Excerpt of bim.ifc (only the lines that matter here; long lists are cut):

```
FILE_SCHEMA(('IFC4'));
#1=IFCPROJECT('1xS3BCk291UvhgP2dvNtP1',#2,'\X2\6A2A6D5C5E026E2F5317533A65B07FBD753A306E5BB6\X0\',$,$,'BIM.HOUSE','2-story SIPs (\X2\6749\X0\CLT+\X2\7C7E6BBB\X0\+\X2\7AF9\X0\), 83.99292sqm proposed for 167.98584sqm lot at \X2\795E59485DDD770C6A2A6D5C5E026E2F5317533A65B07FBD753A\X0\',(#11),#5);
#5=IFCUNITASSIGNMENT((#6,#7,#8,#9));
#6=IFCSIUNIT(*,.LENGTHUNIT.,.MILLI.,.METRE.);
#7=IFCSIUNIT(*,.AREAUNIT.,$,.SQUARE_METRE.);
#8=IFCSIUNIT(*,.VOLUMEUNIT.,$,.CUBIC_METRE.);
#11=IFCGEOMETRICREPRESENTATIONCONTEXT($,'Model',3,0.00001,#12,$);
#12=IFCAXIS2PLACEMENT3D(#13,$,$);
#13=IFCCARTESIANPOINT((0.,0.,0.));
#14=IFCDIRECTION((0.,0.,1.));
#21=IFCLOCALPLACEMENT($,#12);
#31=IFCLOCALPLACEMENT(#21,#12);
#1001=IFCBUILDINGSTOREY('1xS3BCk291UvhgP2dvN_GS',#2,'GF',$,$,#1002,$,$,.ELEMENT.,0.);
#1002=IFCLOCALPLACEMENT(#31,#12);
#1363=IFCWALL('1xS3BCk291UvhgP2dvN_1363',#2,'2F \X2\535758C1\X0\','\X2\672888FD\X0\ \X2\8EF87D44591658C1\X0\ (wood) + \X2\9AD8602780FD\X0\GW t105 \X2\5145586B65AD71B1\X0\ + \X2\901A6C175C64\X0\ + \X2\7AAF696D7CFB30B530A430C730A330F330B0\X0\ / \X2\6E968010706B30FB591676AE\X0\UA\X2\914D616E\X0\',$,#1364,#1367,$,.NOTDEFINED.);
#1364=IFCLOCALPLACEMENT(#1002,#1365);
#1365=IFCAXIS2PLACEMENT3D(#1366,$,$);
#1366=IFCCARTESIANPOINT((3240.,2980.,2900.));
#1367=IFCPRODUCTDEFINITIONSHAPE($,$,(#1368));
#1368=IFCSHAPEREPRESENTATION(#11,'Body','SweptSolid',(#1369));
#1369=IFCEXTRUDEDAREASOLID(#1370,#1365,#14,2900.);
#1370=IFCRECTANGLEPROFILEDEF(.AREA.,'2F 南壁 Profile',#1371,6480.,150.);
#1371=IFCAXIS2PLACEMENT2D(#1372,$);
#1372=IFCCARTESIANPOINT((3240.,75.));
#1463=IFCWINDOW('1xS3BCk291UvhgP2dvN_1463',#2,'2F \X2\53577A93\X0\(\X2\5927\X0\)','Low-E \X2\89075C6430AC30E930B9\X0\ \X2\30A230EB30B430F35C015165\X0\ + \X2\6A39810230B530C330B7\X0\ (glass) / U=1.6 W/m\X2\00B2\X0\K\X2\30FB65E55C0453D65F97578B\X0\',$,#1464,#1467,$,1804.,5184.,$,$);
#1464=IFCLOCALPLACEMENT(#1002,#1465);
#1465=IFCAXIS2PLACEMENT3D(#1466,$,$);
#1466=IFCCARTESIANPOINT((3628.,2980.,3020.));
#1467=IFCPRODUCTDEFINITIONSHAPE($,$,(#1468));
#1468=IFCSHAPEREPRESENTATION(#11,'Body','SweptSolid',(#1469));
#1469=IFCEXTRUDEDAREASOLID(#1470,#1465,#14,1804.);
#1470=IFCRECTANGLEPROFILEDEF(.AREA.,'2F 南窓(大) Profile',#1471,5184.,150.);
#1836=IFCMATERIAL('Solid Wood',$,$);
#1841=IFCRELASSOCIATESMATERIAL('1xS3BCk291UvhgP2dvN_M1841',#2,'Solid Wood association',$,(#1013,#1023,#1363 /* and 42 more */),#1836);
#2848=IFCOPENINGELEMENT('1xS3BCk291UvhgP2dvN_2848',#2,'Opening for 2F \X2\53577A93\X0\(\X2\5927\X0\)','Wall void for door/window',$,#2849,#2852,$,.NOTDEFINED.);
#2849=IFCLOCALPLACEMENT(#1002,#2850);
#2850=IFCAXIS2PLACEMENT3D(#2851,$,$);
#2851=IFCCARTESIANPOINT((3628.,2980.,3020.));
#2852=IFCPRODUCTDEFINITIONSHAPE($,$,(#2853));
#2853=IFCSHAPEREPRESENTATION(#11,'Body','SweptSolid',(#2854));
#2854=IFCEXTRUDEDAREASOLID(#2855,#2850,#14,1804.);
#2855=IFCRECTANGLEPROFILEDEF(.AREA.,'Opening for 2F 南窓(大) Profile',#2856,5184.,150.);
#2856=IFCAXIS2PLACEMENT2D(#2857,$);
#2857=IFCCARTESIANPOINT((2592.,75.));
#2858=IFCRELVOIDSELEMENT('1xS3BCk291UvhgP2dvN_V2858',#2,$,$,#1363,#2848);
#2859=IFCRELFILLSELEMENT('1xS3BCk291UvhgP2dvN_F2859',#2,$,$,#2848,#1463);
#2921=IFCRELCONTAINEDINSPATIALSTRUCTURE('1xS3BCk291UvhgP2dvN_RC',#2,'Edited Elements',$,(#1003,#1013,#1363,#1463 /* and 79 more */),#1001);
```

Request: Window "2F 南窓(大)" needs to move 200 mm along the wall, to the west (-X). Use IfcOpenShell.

```python
import ifcopenshell
import ifcopenshell.api.geometry
import ifcopenshell.util.placement

model = ifcopenshell.open("bim.ifc")

window = model.by_guid("1xS3BCk291UvhgP2dvN_1463")
opening = window.FillsVoids[0].RelatingOpeningElement
wall = opening.VoidsElements[0].RelatingBuildingElement

wall_matrix = ifcopenshell.util.placement.get_local_placement(wall.ObjectPlacement)
shift = wall_matrix[:3, 0] * -200.0
before = ifcopenshell.util.placement.get_local_placement(window.ObjectPlacement)[:3, 3].copy()

# The window is not placed relative to its opening, so move both.
for product in (opening, window):
    matrix = ifcopenshell.util.placement.get_local_placement(product.ObjectPlacement)
    matrix[:3, 3] += shift
    ifcopenshell.api.geometry.edit_object_placement(model, product=product, matrix=matrix, is_si=False)

after = ifcopenshell.util.placement.get_local_placement(window.ObjectPlacement)[:3, 3]
print("window moved by", (after - before).round(3) + 0.0)

model.write("bim-out.ifc")
```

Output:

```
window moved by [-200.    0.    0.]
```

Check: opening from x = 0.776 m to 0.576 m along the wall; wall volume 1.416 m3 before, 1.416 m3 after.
